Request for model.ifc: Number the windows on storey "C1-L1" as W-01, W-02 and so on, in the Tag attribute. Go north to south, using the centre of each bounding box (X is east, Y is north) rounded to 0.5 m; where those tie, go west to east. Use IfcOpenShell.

First a look at what the model holds.

```python
import ifcopenshell
import ifcopenshell.util.element
import ifcopenshell.util.placement

model = ifcopenshell.open("model.ifc")
print(model.schema)
storey = next(s for s in model.by_type("IfcBuildingStorey") if s.Name == "C1-L1")
windows = [e for e in ifcopenshell.util.element.get_decomposition(storey) if e.is_a("IfcWindow")]
for e in sorted(windows, key=lambda e: e.id()):
    origin = ifcopenshell.util.placement.get_local_placement(e.ObjectPlacement)[:3, 3]
    print(e.id(), e.Tag, e.Name, origin.round(2) + 0.0, sep=" | ")
```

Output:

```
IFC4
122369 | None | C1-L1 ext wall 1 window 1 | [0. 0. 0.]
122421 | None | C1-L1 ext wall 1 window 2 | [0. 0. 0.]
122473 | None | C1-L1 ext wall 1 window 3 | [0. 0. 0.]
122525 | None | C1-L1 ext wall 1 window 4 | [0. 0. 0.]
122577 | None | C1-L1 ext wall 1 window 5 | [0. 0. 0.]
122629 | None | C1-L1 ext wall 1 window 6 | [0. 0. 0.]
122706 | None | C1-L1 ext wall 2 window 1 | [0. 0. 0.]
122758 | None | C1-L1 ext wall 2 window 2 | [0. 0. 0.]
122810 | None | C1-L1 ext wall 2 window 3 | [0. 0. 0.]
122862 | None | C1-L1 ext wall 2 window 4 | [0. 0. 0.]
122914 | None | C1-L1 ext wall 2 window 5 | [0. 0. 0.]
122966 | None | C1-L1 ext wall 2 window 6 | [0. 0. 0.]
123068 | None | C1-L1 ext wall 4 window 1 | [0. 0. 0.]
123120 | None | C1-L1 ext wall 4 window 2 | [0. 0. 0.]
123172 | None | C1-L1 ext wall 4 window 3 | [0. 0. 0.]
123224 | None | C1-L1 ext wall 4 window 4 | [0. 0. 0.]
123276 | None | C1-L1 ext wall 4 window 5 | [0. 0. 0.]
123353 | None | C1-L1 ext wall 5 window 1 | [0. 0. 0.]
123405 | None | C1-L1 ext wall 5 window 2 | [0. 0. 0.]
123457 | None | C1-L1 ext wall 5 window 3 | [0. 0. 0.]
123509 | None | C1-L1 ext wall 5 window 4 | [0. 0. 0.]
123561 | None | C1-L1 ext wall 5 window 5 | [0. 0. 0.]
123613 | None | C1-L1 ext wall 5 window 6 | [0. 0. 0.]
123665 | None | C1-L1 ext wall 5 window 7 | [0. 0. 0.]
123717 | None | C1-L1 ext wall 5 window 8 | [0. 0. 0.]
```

```python
import ifcopenshell
import ifcopenshell.geom
import ifcopenshell.util.element
import ifcopenshell.util.shape

model = ifcopenshell.open("model.ifc")
settings = ifcopenshell.geom.settings()
settings.set("use-world-coords", True)


def centre(element):
    shape = ifcopenshell.geom.create_shape(settings, element)
    return ifcopenshell.util.shape.get_bbox_centroid(shape.geometry)


storey = next(s for s in model.by_type("IfcBuildingStorey") if s.Name == "C1-L1")
windows = [e for e in ifcopenshell.util.element.get_decomposition(storey) if e.is_a("IfcWindow")]

# Insertion points can sit at a corner or the storey origin, so sort by the geometry (in metres).
centres = {e: centre(e) for e in windows}
windows.sort(key=lambda e: (-round(centres[e][1] / 0.5), centres[e][0]))

for i, e in enumerate(windows, start=1):
    number = f"W-{i:02d}"
    e.Tag = number
    print(e.id(), number)

model.write("model_rev.ifc")
```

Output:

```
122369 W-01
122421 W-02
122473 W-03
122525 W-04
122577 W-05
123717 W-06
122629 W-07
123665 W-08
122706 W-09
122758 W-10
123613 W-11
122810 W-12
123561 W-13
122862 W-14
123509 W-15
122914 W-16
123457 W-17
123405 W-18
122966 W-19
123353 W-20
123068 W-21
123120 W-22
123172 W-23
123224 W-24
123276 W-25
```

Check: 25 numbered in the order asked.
